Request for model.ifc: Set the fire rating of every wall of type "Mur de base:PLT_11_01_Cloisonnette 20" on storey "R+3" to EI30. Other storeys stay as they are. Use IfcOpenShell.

First a look at what the model holds.

```python
import ifcopenshell
import ifcopenshell.util.element

model = ifcopenshell.open("model.ifc")
print(model.schema)
storey = next(s for s in model.by_type("IfcBuildingStorey") if s.Name == "R+3")
walls = [e for e in ifcopenshell.util.element.get_decomposition(storey) if e.is_a("IfcWall")]
seen = {}
for e in walls:
    element_type = ifcopenshell.util.element.get_type(e)
    key = (element_type.Name if element_type != e and element_type else None, ifcopenshell.util.element.get_pset(e, "Pset_WallCommon", "FireRating"))
    seen[key] = seen.get(key, 0) + 1
for (name, value), count in sorted(seen.items(), key=str):
    print(count, "x", name, "|", value)
```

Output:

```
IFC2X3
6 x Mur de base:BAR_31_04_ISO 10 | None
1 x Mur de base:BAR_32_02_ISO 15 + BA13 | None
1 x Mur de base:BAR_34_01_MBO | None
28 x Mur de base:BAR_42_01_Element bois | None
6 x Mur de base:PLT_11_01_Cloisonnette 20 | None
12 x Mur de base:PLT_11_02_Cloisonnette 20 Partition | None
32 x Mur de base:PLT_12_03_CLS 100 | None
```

```python
import ifcopenshell
import ifcopenshell.api.pset
import ifcopenshell.util.element

model = ifcopenshell.open("model.ifc")

storey = next(s for s in model.by_type("IfcBuildingStorey") if s.Name == "R+3")
walls = [e for e in ifcopenshell.util.element.get_decomposition(storey) if e.is_a("IfcWall")]

count = 0
for e in walls:
    element_type = ifcopenshell.util.element.get_type(e)
    if element_type in (None, e) or element_type.Name != "Mur de base:PLT_11_01_Cloisonnette 20":
        continue
    # add_pset returns the element's existing set when there is one.
    pset = ifcopenshell.api.pset.add_pset(model, product=e, name="Pset_WallCommon")
    ifcopenshell.api.pset.edit_pset(model, pset=pset, properties={"FireRating": "EI30"})
    count += 1

print(count, "walls updated")

model.write("model_updated.ifc")
```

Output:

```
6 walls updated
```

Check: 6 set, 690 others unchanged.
